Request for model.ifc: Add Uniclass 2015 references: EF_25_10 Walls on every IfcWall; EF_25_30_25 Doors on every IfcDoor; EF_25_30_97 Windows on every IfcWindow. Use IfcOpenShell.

First a look at what the model holds.

```python
import ifcopenshell

model = ifcopenshell.open("model.ifc")
print(model.schema)
print("classifications:", [c.Name for c in model.by_type("IfcClassification")])
for ifc_class in ("IfcDoor", "IfcRoof", "IfcStair", "IfcWall", "IfcWindow"):
    print(ifc_class, len(model.by_type(ifc_class)))
```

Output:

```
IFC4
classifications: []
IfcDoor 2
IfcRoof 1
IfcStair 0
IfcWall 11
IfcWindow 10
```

```python
import ifcopenshell
import ifcopenshell.api.classification

model = ifcopenshell.open("model.ifc")

system = ifcopenshell.api.classification.add_classification(model, classification="Uniclass 2015")

codes = {
    "IfcWall": ("EF_25_10", "Walls"),
    "IfcDoor": ("EF_25_30_25", "Doors"),
    "IfcWindow": ("EF_25_30_97", "Windows"),
}
for ifc_class, (code, name) in codes.items():
    products = model.by_type(ifc_class)
    ifcopenshell.api.classification.add_reference(
        model, products=products, classification=system, identification=code, name=name
    )
    print(code, len(products))

model.write("model_rev.ifc")
```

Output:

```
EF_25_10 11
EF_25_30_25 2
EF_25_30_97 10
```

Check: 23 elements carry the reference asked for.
